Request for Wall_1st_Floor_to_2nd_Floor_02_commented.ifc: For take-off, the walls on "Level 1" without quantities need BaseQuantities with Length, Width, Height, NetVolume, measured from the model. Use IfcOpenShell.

First a look at what the model holds.

```python
import ifcopenshell
import ifcopenshell.util.element
import ifcopenshell.util.unit

model = ifcopenshell.open("Wall_1st_Floor_to_2nd_Floor_02_commented.ifc")
print(model.schema)
for unit_type in ("LENGTHUNIT", "AREAUNIT", "VOLUMEUNIT"):
    print(unit_type, ifcopenshell.util.unit.calculate_unit_scale(model, unit_type))
storey = next(s for s in model.by_type("IfcBuildingStorey") if s.Name == "Level 1")
walls = [e for e in ifcopenshell.util.element.get_decomposition(storey) if e.is_a("IfcWall")]
for e in sorted(walls, key=lambda e: e.id()):
    print(e.id(), e.is_a(), e.Name, list(ifcopenshell.util.element.get_psets(e, qtos_only=True)), sep=" | ")
```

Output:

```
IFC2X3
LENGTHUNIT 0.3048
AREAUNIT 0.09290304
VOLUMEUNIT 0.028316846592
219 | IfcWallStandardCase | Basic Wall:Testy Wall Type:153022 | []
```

```python
import ifcopenshell
import ifcopenshell.api.pset
import ifcopenshell.geom
import ifcopenshell.util.element
import ifcopenshell.util.shape
import ifcopenshell.util.unit

model = ifcopenshell.open("Wall_1st_Floor_to_2nd_Floor_02_commented.ifc")
unit_scale = ifcopenshell.util.unit.calculate_unit_scale(model)
volume_scale = ifcopenshell.util.unit.calculate_unit_scale(model, "VOLUMEUNIT")
settings = ifcopenshell.geom.settings()

storey = next(s for s in model.by_type("IfcBuildingStorey") if s.Name == "Level 1")
walls = [e for e in ifcopenshell.util.element.get_decomposition(storey) if e.is_a("IfcWall")]

for e in sorted(walls, key=lambda e: e.id()):
    if ifcopenshell.util.element.get_psets(e, qtos_only=True, should_inherit=False):
        continue
    # Geometry comes back in metres, in the element's own axes.
    shape = ifcopenshell.geom.create_shape(settings, e)
    values = {
        "Length": ifcopenshell.util.shape.get_x(shape.geometry) / unit_scale,
        "Width": ifcopenshell.util.shape.get_y(shape.geometry) / unit_scale,
        "Height": ifcopenshell.util.shape.get_z(shape.geometry) / unit_scale,
        "NetVolume": ifcopenshell.util.shape.get_volume(shape.geometry) / volume_scale,
    }
    qto = ifcopenshell.api.pset.add_qto(model, product=e, name="BaseQuantities")
    ifcopenshell.api.pset.edit_qto(model, qto=qto, properties=values)
    print(e.id(), {k: round(v, 3) for k, v in values.items()})

model.write("Wall_1st_Floor_to_2nd_Floor_02_commented_updated.ifc")
```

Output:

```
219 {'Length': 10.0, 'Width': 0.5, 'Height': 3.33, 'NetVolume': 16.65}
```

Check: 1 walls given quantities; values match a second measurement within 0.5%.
